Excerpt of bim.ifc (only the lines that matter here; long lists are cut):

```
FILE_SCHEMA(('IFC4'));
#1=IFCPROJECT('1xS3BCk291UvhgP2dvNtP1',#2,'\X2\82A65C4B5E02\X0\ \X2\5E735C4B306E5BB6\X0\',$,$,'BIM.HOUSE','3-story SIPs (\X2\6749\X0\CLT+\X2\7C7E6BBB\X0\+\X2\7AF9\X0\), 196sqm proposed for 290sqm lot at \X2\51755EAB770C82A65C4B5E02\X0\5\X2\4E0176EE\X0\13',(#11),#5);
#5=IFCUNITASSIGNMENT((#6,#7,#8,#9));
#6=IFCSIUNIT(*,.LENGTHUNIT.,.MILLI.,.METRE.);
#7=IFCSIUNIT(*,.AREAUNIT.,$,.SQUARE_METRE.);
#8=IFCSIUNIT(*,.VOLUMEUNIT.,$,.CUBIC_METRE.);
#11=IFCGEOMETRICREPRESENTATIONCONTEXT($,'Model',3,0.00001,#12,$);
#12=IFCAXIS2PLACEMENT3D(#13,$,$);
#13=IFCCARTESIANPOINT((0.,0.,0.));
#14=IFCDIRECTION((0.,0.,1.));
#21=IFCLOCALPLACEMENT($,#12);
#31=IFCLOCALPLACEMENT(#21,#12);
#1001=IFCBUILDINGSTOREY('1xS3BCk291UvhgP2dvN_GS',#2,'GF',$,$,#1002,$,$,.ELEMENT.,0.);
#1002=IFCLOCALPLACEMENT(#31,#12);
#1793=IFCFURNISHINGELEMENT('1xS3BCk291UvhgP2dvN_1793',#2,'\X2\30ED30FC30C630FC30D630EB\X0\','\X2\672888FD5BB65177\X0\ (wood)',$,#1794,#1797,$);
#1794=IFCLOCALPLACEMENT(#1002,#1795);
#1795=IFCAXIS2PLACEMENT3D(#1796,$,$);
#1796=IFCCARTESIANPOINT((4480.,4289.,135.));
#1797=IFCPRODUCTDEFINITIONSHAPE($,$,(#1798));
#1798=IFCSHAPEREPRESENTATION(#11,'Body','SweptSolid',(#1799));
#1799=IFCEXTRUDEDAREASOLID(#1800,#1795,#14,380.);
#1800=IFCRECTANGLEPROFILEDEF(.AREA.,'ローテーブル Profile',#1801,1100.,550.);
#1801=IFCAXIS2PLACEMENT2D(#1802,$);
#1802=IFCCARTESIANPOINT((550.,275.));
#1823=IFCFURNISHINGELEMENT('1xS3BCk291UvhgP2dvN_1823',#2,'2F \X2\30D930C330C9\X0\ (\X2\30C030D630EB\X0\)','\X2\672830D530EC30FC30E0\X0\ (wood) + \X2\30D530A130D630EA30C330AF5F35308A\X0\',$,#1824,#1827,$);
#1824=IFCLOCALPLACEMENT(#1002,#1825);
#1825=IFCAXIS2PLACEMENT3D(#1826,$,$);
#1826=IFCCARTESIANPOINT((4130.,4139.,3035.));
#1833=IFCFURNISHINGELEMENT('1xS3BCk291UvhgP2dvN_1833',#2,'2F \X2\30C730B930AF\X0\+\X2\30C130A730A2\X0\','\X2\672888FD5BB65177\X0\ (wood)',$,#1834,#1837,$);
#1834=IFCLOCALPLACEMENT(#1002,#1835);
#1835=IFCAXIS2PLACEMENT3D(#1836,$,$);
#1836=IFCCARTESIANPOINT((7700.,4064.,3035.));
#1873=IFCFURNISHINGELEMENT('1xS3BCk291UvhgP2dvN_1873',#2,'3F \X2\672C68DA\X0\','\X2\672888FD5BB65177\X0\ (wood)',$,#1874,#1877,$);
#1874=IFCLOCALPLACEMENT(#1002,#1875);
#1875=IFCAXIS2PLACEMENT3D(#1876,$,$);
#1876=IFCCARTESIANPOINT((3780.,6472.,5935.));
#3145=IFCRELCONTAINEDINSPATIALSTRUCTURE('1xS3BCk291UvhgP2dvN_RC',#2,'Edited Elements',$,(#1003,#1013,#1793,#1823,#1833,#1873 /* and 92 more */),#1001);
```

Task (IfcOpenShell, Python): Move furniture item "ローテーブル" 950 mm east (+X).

```python
import ifcopenshell
import ifcopenshell.api.geometry
import ifcopenshell.util.placement
import ifcopenshell.util.unit

model = ifcopenshell.open("bim.ifc")
unit_scale = ifcopenshell.util.unit.calculate_unit_scale(model)

item = model.by_guid("1xS3BCk291UvhgP2dvN_1793")
matrix = ifcopenshell.util.placement.get_local_placement(item.ObjectPlacement)
matrix[0, 3] += 0.95 / unit_scale
ifcopenshell.api.geometry.edit_object_placement(model, product=item, matrix=matrix, is_si=False)

print(ifcopenshell.util.placement.get_local_placement(item.ObjectPlacement).round(3) + 0.0)

model.write("bim_v2.ifc")
```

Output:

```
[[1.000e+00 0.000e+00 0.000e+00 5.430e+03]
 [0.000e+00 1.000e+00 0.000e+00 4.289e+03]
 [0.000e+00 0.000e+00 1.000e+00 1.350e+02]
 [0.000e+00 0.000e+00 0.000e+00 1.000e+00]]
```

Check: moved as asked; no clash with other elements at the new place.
